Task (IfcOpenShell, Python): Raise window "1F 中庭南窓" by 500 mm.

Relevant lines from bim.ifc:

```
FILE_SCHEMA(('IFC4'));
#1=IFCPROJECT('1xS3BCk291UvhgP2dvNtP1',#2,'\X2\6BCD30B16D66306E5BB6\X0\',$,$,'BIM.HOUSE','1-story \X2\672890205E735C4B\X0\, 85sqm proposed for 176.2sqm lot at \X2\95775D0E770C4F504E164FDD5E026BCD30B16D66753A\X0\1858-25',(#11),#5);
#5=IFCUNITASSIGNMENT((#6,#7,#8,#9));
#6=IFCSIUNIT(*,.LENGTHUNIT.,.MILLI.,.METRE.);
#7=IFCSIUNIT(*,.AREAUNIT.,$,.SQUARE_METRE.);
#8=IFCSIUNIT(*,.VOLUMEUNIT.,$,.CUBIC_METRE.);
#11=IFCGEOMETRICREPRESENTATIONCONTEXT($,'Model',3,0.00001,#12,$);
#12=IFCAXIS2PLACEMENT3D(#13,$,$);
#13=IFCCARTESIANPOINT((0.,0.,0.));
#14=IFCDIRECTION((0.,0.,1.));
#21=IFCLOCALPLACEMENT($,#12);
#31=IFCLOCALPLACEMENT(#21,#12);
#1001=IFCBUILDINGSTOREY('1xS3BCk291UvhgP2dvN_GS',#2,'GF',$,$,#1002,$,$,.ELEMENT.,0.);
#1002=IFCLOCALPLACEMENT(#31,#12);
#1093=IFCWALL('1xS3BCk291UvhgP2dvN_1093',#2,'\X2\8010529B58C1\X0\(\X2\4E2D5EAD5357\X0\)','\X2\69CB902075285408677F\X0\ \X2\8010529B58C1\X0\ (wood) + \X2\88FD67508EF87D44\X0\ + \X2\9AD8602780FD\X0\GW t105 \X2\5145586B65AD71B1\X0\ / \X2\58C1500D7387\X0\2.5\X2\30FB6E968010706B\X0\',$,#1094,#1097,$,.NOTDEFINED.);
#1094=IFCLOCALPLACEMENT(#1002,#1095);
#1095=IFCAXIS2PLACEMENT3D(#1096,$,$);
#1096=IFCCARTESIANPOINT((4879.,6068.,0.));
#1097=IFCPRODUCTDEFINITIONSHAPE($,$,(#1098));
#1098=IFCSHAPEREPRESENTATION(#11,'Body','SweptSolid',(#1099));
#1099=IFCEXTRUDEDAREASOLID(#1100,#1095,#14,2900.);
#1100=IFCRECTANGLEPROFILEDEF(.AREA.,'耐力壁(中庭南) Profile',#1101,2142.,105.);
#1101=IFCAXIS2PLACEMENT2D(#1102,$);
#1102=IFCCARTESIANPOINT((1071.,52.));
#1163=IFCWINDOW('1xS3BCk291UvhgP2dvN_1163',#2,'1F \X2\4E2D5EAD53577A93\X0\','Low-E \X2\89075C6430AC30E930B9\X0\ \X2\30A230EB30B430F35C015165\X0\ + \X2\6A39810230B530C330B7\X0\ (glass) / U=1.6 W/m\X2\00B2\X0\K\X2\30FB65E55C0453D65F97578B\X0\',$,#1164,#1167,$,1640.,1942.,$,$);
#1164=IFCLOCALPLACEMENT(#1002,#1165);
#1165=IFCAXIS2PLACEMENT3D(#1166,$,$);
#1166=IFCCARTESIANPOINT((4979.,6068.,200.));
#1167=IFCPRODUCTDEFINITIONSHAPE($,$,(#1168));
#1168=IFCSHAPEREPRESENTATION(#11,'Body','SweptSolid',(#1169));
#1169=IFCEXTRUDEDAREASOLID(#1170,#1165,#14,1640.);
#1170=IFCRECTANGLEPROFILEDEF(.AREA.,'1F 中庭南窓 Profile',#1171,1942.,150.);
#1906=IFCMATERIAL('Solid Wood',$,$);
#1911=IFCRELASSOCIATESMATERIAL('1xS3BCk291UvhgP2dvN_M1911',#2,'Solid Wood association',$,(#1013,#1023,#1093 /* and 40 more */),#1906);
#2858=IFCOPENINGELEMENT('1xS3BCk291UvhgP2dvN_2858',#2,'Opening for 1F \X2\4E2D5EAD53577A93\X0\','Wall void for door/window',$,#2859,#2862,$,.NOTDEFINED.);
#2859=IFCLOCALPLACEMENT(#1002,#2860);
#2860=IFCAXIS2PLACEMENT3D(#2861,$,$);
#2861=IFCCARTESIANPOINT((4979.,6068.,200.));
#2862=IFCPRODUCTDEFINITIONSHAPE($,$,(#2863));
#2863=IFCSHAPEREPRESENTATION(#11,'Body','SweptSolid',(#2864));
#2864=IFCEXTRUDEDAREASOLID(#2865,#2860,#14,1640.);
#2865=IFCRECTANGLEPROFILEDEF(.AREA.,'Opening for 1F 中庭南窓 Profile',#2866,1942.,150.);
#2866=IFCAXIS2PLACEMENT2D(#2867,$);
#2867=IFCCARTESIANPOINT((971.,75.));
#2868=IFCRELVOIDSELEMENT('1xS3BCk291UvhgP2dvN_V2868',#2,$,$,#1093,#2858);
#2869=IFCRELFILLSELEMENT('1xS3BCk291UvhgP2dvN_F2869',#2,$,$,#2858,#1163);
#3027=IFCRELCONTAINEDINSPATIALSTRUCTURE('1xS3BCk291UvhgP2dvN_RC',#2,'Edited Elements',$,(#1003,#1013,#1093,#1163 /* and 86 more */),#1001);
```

```python
import numpy as np
import ifcopenshell
import ifcopenshell.api.geometry
import ifcopenshell.util.placement
import ifcopenshell.util.unit

model = ifcopenshell.open("bim.ifc")
unit_scale = ifcopenshell.util.unit.calculate_unit_scale(model)

window = model.by_guid("1xS3BCk291UvhgP2dvN_1163")
opening = window.FillsVoids[0].RelatingOpeningElement
dz = 0.5 / unit_scale

shift = np.array([0.0, 0.0, dz])
# The window is not placed relative to its opening, so move both.
for product in (opening, window):
    matrix = ifcopenshell.util.placement.get_local_placement(product.ObjectPlacement)
    matrix[:3, 3] += shift
    ifcopenshell.api.geometry.edit_object_placement(model, product=product, matrix=matrix, is_si=False)

print(f"moved by {dz * unit_scale:+.3f} m")

model.write("bim-out.ifc")
```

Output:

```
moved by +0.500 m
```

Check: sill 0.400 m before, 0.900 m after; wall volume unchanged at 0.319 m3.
